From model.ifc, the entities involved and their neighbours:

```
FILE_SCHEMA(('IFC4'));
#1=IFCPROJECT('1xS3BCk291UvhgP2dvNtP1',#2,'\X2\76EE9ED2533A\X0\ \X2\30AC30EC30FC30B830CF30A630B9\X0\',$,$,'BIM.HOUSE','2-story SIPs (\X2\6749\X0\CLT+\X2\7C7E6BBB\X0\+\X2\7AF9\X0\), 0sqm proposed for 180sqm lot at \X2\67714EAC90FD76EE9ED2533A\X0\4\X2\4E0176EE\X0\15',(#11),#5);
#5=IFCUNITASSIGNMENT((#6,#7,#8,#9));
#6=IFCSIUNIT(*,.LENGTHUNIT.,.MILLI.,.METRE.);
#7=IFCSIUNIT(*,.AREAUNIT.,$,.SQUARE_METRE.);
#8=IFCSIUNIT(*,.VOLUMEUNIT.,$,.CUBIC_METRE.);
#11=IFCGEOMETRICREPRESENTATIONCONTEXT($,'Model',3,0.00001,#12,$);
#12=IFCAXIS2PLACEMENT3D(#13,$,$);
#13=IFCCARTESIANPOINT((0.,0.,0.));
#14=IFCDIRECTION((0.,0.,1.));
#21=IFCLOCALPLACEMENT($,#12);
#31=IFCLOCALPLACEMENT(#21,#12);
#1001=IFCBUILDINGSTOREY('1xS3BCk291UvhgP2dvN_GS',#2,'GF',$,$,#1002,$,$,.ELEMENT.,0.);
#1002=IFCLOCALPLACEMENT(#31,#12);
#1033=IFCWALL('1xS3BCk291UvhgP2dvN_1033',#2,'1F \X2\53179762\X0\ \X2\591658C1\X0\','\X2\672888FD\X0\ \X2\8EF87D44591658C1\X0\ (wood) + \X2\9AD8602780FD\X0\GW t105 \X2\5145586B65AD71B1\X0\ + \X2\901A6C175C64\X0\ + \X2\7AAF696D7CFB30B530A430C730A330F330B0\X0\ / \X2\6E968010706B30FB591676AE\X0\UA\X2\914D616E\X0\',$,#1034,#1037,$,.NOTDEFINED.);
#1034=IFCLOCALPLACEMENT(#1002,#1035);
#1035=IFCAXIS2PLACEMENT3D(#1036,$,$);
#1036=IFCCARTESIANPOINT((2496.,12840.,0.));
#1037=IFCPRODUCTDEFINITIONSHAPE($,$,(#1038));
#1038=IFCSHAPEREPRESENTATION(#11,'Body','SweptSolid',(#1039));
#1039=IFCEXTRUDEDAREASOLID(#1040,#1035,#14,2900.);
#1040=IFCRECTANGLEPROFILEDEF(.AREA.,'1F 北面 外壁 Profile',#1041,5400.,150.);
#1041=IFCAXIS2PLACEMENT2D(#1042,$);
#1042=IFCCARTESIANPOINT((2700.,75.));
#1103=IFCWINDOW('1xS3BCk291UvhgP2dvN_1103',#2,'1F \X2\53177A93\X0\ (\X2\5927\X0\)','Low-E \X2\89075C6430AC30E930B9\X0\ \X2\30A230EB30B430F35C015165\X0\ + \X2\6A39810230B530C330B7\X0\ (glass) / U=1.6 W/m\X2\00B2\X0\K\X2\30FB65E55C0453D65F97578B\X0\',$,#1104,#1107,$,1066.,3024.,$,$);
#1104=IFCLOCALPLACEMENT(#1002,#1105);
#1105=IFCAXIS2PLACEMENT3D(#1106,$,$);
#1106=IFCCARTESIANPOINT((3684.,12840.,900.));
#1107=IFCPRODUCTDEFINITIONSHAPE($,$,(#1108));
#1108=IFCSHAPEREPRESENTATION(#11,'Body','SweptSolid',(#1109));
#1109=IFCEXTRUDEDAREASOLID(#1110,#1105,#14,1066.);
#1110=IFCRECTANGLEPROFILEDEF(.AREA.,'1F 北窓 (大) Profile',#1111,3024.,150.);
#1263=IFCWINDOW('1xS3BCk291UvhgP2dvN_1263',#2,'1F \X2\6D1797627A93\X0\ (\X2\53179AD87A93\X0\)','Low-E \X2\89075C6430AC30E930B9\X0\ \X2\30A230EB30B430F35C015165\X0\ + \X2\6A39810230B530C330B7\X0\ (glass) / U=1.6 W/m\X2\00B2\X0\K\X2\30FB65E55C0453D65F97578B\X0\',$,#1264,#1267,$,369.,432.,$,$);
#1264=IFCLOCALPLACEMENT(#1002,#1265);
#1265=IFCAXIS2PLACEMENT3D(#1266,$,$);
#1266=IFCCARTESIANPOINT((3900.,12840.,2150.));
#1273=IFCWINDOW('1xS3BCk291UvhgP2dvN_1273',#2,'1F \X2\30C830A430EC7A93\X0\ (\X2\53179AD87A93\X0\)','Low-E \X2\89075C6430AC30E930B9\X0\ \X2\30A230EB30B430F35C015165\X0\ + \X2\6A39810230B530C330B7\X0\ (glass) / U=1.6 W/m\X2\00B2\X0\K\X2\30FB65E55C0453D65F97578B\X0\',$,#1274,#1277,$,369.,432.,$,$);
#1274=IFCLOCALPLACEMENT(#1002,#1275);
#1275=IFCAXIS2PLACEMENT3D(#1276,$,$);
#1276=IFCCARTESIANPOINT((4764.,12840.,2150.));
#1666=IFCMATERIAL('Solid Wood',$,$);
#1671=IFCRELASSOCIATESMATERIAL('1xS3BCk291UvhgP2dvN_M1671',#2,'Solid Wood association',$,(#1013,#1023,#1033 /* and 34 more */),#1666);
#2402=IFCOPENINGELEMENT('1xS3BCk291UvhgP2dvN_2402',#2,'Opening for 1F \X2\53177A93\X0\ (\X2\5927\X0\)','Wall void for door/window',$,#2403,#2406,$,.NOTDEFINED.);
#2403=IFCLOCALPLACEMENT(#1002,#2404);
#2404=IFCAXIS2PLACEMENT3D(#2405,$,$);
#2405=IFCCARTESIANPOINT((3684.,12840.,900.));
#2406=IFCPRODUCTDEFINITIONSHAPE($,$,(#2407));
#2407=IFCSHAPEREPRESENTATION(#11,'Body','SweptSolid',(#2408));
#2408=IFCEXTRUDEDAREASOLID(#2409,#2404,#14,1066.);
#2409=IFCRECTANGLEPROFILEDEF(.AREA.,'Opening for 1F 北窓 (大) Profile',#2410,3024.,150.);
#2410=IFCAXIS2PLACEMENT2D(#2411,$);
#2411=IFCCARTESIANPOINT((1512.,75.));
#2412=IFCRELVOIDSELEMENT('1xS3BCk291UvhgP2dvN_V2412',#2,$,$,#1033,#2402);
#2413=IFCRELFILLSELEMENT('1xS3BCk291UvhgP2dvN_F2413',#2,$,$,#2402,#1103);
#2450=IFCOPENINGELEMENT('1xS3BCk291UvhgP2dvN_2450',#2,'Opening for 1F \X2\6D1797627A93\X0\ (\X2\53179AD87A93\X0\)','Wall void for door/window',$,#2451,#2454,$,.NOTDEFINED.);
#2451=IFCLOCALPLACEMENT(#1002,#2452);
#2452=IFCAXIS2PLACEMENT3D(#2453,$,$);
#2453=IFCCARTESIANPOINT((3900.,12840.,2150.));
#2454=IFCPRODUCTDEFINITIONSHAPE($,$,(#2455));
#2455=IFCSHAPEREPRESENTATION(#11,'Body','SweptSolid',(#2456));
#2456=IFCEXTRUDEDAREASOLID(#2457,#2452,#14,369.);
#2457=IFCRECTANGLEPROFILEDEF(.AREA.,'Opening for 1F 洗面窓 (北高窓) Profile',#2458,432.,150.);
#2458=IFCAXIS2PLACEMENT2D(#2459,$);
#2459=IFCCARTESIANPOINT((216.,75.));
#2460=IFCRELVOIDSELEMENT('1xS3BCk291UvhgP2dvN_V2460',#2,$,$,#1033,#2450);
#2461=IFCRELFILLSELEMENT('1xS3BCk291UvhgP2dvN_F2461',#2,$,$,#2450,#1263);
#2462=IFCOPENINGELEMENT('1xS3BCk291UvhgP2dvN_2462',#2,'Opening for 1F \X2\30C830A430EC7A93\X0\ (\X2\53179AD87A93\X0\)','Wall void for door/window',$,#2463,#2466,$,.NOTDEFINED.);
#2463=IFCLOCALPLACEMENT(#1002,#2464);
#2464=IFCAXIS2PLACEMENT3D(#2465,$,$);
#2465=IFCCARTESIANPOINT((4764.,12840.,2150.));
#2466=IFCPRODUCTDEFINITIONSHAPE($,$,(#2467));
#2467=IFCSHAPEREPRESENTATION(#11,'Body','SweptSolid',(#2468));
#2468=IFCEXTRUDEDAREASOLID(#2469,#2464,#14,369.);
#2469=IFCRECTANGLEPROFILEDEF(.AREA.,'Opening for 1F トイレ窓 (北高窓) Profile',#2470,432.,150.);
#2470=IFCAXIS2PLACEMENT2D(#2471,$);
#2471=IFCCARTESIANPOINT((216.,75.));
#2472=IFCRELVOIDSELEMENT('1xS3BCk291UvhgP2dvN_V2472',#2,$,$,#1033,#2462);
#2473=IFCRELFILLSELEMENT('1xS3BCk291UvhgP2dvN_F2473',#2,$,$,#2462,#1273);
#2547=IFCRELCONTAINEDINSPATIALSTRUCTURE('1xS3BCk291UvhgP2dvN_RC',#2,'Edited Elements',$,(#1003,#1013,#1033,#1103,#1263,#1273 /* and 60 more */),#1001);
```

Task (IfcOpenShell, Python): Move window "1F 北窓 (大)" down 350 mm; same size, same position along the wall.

```python
import numpy as np
import ifcopenshell
import ifcopenshell.api.geometry
import ifcopenshell.util.placement
import ifcopenshell.util.unit

model = ifcopenshell.open("model.ifc")
unit_scale = ifcopenshell.util.unit.calculate_unit_scale(model)

window = model.by_guid("1xS3BCk291UvhgP2dvN_1103")
opening = window.FillsVoids[0].RelatingOpeningElement
dz = -0.35 / unit_scale

shift = np.array([0.0, 0.0, dz])
# The window is not placed relative to its opening, so move both.
for product in (opening, window):
    matrix = ifcopenshell.util.placement.get_local_placement(product.ObjectPlacement)
    matrix[:3, 3] += shift
    ifcopenshell.api.geometry.edit_object_placement(model, product=product, matrix=matrix, is_si=False)

print(f"moved by {dz * unit_scale:+.3f} m")

model.write("model_edited.ifc")
```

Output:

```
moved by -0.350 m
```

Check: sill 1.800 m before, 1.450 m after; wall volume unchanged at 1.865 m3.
